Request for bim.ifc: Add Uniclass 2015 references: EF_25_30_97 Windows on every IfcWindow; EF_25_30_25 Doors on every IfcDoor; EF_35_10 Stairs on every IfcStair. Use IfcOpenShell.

First a look at what the model holds.

```python
import ifcopenshell

model = ifcopenshell.open("bim.ifc")
print(model.schema)
print("classifications:", [c.Name for c in model.by_type("IfcClassification")])
for ifc_class in ("IfcDoor", "IfcRoof", "IfcStair", "IfcWall", "IfcWindow"):
    print(ifc_class, len(model.by_type(ifc_class)))
```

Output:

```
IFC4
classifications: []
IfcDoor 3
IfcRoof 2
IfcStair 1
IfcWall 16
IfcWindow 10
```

```python
import ifcopenshell
import ifcopenshell.api.classification

model = ifcopenshell.open("bim.ifc")

system = ifcopenshell.api.classification.add_classification(model, classification="Uniclass 2015")

codes = {
    "IfcWindow": ("EF_25_30_97", "Windows"),
    "IfcDoor": ("EF_25_30_25", "Doors"),
    "IfcStair": ("EF_35_10", "Stairs"),
}
for ifc_class, (code, name) in codes.items():
    products = model.by_type(ifc_class)
    ifcopenshell.api.classification.add_reference(
        model, products=products, classification=system, identification=code, name=name
    )
    print(code, len(products))

model.write("bim_edited.ifc")
```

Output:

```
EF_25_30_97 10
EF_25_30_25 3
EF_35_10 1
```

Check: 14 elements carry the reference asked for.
